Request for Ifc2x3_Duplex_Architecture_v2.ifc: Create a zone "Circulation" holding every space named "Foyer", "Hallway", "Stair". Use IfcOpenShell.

First a look at what the model holds.

```python
import ifcopenshell

model = ifcopenshell.open("Ifc2x3_Duplex_Architecture_v2.ifc")
print(model.schema)
seen = {}
for space in model.by_type("IfcSpace"):
    seen[space.LongName] = seen.get(space.LongName, 0) + 1
for name, count in sorted(seen.items(), key=str):
    print(count, "x", name)
print("zones:", [z.Name for z in model.by_type("IfcZone")][:20])
```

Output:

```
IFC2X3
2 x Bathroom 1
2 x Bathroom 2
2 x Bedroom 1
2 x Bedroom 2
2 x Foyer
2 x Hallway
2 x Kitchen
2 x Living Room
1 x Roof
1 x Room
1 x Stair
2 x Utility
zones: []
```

```python
import ifcopenshell
import ifcopenshell.api.group
import ifcopenshell.api.root

model = ifcopenshell.open("Ifc2x3_Duplex_Architecture_v2.ifc")

names = {"Foyer", "Hallway", "Stair"}
spaces = [s for s in model.by_type("IfcSpace") if s.LongName in names]

zone = ifcopenshell.api.root.create_entity(model, ifc_class="IfcZone", name="Circulation")
ifcopenshell.api.group.assign_group(model, products=spaces, group=zone)
print(len(spaces), "spaces in", zone.Name)

model.write("Ifc2x3_Duplex_Architecture_v2-out.ifc")
```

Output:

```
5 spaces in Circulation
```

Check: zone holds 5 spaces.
